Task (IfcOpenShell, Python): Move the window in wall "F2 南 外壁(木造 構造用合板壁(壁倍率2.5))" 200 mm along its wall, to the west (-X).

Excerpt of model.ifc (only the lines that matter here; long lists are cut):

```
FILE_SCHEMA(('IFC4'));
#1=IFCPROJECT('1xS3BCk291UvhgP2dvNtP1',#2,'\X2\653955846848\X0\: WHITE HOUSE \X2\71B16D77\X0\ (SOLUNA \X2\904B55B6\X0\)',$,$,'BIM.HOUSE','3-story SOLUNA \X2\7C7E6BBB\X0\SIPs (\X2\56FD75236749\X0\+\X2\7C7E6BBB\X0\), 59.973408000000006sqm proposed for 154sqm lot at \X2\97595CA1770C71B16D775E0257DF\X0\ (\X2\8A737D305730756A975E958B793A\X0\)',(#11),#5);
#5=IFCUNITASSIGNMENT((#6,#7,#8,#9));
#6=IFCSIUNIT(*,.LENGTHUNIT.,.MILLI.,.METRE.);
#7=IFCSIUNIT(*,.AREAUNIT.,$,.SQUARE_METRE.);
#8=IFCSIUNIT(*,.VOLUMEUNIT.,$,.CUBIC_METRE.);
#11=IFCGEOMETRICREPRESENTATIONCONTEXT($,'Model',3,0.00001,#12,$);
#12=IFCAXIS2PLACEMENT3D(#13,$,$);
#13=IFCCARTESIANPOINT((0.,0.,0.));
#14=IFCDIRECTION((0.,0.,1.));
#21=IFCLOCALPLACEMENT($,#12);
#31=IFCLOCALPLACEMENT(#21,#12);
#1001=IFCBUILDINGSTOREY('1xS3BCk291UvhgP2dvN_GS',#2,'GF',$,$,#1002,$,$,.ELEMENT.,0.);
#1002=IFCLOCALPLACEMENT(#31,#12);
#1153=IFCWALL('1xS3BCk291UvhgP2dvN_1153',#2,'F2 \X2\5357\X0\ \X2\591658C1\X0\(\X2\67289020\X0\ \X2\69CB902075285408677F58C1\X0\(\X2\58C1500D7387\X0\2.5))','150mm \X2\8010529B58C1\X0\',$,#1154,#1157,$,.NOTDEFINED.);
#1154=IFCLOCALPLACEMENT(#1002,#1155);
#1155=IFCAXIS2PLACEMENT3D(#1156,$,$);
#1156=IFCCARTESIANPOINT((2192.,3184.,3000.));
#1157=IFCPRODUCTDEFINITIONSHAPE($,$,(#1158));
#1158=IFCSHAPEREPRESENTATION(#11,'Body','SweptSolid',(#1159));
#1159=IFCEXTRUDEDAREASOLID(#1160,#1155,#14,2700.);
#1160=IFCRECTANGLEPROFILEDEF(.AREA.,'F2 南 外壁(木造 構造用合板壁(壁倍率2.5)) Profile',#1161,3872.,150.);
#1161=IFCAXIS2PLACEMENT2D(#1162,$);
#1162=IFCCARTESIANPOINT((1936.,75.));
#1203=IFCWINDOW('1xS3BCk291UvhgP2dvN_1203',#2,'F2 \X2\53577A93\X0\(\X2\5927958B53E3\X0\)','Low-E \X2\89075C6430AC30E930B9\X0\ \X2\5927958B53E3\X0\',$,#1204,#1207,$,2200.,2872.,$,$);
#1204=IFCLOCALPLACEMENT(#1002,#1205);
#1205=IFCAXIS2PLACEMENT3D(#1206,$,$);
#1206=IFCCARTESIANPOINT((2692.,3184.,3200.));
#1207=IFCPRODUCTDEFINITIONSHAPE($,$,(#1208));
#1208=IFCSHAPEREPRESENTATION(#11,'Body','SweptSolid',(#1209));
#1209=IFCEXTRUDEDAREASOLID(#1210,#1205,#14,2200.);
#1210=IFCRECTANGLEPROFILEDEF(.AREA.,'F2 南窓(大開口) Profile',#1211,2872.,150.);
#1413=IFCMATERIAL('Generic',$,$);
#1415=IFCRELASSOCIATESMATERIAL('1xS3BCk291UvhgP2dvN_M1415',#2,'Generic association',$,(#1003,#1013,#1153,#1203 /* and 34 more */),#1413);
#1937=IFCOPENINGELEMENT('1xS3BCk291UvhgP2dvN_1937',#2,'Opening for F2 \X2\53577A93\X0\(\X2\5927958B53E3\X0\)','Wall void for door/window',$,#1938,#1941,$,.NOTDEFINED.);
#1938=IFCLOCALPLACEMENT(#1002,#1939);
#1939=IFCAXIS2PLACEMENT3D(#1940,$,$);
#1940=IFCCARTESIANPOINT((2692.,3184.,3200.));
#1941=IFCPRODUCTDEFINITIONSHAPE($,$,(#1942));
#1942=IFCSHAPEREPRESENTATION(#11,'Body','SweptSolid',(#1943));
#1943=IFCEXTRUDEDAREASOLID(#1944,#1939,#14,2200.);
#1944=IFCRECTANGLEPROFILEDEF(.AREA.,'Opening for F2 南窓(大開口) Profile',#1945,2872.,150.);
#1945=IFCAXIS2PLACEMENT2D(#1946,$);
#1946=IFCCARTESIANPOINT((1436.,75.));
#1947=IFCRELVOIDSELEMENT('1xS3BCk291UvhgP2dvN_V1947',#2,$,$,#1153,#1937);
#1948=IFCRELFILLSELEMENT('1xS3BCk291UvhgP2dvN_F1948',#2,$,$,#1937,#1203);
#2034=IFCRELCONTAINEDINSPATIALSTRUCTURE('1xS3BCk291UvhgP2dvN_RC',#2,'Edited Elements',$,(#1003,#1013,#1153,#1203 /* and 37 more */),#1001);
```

```python
import ifcopenshell
import ifcopenshell.api.geometry
import ifcopenshell.util.placement

model = ifcopenshell.open("model.ifc")

window = model.by_guid("1xS3BCk291UvhgP2dvN_1203")
opening = window.FillsVoids[0].RelatingOpeningElement
wall = opening.VoidsElements[0].RelatingBuildingElement

wall_matrix = ifcopenshell.util.placement.get_local_placement(wall.ObjectPlacement)
shift = wall_matrix[:3, 0] * -200.0
before = ifcopenshell.util.placement.get_local_placement(window.ObjectPlacement)[:3, 3].copy()

# The window is not placed relative to its opening, so move both.
for product in (opening, window):
    matrix = ifcopenshell.util.placement.get_local_placement(product.ObjectPlacement)
    matrix[:3, 3] += shift
    ifcopenshell.api.geometry.edit_object_placement(model, product=product, matrix=matrix, is_si=False)

after = ifcopenshell.util.placement.get_local_placement(window.ObjectPlacement)[:3, 3]
print("window moved by", (after - before).round(3) + 0.0)

model.write("model-out.ifc")
```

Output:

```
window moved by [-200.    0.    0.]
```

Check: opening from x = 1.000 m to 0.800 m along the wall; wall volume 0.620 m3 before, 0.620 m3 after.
